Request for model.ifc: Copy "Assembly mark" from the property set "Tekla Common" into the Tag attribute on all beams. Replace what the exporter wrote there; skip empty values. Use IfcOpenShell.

First a look at what the model holds.

```python
import ifcopenshell
import ifcopenshell.util.element

model = ifcopenshell.open("model.ifc")
print(model.schema)
beams = model.by_type("IfcBeam")
print(len(beams), "beams")
for e in beams[:8]:
    source = ifcopenshell.util.element.get_pset(e, "Tekla Common", "Assembly mark")
    target = e.Tag
    print(e.id(), repr(source), repr(target), sep=" | ")
```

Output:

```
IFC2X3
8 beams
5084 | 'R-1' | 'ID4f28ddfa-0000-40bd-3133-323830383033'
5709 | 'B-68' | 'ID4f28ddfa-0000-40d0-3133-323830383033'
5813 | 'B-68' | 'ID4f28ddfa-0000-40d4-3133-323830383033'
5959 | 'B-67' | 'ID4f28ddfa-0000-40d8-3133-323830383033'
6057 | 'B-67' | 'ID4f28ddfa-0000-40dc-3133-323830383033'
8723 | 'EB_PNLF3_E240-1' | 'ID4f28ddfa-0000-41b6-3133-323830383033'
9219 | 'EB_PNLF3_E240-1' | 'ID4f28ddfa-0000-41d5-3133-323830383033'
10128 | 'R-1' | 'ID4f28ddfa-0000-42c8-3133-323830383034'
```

```python
import ifcopenshell
import ifcopenshell.util.element

model = ifcopenshell.open("model.ifc")

count = 0
for e in model.by_type("IfcBeam"):
    value = ifcopenshell.util.element.get_pset(e, "Tekla Common", "Assembly mark")
    current = e.Tag
    if not value or not value.strip() or current == value:
        continue
    e.Tag = value
    count += 1

print(count, "beams updated")

model.write("model_updated.ifc")
```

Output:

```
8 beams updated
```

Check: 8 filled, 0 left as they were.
